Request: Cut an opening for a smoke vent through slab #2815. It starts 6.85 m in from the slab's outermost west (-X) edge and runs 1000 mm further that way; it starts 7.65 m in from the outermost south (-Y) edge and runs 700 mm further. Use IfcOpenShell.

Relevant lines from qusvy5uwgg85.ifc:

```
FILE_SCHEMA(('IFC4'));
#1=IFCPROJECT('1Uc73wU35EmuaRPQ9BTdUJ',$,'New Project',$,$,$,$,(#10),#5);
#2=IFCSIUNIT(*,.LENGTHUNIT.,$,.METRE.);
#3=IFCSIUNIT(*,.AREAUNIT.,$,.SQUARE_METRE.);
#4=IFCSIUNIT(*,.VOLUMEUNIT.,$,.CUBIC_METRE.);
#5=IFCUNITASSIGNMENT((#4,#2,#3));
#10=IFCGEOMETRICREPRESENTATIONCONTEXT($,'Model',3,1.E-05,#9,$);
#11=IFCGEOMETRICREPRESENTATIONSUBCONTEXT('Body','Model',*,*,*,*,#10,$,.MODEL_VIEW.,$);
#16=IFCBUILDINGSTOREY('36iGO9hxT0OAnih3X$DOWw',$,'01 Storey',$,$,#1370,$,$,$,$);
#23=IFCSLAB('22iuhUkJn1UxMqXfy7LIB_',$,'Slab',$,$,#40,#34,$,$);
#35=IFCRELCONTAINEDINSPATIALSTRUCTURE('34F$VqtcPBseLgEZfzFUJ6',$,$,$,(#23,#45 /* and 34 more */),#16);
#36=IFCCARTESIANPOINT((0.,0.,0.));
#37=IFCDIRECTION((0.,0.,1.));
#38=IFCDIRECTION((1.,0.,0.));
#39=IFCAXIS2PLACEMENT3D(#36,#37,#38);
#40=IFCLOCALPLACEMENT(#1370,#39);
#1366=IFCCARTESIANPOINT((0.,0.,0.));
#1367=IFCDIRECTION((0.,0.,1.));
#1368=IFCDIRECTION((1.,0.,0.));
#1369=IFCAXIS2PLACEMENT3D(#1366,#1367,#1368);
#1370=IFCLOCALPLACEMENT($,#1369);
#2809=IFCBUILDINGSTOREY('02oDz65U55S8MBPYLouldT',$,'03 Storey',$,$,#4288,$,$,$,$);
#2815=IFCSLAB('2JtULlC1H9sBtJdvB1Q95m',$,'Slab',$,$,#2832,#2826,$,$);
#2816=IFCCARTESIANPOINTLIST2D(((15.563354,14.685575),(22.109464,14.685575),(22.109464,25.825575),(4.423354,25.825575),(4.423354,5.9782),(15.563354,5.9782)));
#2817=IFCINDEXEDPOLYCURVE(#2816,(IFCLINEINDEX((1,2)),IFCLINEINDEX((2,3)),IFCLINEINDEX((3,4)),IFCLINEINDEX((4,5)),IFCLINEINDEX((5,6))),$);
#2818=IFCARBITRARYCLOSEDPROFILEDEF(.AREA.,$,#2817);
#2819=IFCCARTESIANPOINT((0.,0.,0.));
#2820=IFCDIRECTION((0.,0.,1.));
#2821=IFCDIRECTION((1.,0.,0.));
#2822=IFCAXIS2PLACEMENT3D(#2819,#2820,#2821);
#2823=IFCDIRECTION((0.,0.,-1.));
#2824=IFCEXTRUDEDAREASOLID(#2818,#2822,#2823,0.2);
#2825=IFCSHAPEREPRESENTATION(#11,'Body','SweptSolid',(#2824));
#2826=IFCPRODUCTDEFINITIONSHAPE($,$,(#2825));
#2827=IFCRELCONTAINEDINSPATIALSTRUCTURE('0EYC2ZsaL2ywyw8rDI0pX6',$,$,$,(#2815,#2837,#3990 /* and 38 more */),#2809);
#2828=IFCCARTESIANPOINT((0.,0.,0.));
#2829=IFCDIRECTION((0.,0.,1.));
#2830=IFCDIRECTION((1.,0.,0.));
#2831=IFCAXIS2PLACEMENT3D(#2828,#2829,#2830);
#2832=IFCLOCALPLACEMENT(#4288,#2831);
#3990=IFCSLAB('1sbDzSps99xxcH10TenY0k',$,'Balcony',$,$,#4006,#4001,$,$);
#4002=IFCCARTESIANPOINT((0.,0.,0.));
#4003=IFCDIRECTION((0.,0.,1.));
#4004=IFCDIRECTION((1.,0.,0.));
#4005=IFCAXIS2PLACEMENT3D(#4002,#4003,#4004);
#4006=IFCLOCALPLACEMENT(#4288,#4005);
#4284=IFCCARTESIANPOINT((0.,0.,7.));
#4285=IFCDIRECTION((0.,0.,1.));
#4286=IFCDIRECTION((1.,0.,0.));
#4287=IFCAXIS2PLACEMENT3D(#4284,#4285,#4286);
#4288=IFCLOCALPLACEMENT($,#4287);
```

```python
import numpy as np
import ifcopenshell
import ifcopenshell.api.feature
import ifcopenshell.api.geometry
import ifcopenshell.api.root
import ifcopenshell.geom
import ifcopenshell.util.placement
import ifcopenshell.util.representation
import ifcopenshell.util.shape
import ifcopenshell.util.unit

model = ifcopenshell.open("qusvy5uwgg85.ifc")
unit_scale = ifcopenshell.util.unit.calculate_unit_scale(model)
settings = ifcopenshell.geom.settings()


def volume(element):
    """Net volume in cubic metres, openings subtracted."""
    shape = ifcopenshell.geom.create_shape(settings, element)
    return ifcopenshell.util.shape.get_volume(shape.geometry)


slab = model.by_guid("2JtULlC1H9sBtJdvB1Q95m")
before = volume(slab)

# Extent in the slab's own axes, in metres. The edges named are its -X and -Y sides.
slab_shape = ifcopenshell.geom.create_shape(settings, slab)
vertices = ifcopenshell.util.shape.get_vertices(slab_shape.geometry)
x_min, y_min, bottom = vertices.min(axis=0)
top = vertices[:, 2].max()

opening = ifcopenshell.api.root.create_entity(model, ifc_class="IfcOpeningElement", name="Smoke vent opening", predefined_type="OPENING")
context = ifcopenshell.util.representation.get_context(model, "Model", "Body", "MODEL_VIEW")
width, depth = 1, 0.7
outline = [(0.0, 0.0), (width, 0.0), (width, depth), (0.0, depth), (0.0, 0.0)]
# Overshoot both faces by 50 mm so the cut is clean.
shape = ifcopenshell.api.geometry.add_slab_representation(
    model, context=context, depth=top - bottom + 0.1, polyline=outline
)
ifcopenshell.api.geometry.assign_representation(model, product=opening, representation=shape)

matrix = ifcopenshell.util.placement.get_local_placement(slab.ObjectPlacement)
matrix[:, 3] = matrix @ np.append(np.array([x_min + 6.85, y_min + 7.65, bottom - 0.05]) / unit_scale, 1.0)
ifcopenshell.api.geometry.edit_object_placement(model, product=opening, matrix=matrix, is_si=False)
ifcopenshell.api.feature.add_feature(model, feature=opening, element=slab)

after = volume(slab)

print(f"slab volume {before:.3f} -> {after:.3f} m3")

model.write("qusvy5uwgg85_rev.ifc")
```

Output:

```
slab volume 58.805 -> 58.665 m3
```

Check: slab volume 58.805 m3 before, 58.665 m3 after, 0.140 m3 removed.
